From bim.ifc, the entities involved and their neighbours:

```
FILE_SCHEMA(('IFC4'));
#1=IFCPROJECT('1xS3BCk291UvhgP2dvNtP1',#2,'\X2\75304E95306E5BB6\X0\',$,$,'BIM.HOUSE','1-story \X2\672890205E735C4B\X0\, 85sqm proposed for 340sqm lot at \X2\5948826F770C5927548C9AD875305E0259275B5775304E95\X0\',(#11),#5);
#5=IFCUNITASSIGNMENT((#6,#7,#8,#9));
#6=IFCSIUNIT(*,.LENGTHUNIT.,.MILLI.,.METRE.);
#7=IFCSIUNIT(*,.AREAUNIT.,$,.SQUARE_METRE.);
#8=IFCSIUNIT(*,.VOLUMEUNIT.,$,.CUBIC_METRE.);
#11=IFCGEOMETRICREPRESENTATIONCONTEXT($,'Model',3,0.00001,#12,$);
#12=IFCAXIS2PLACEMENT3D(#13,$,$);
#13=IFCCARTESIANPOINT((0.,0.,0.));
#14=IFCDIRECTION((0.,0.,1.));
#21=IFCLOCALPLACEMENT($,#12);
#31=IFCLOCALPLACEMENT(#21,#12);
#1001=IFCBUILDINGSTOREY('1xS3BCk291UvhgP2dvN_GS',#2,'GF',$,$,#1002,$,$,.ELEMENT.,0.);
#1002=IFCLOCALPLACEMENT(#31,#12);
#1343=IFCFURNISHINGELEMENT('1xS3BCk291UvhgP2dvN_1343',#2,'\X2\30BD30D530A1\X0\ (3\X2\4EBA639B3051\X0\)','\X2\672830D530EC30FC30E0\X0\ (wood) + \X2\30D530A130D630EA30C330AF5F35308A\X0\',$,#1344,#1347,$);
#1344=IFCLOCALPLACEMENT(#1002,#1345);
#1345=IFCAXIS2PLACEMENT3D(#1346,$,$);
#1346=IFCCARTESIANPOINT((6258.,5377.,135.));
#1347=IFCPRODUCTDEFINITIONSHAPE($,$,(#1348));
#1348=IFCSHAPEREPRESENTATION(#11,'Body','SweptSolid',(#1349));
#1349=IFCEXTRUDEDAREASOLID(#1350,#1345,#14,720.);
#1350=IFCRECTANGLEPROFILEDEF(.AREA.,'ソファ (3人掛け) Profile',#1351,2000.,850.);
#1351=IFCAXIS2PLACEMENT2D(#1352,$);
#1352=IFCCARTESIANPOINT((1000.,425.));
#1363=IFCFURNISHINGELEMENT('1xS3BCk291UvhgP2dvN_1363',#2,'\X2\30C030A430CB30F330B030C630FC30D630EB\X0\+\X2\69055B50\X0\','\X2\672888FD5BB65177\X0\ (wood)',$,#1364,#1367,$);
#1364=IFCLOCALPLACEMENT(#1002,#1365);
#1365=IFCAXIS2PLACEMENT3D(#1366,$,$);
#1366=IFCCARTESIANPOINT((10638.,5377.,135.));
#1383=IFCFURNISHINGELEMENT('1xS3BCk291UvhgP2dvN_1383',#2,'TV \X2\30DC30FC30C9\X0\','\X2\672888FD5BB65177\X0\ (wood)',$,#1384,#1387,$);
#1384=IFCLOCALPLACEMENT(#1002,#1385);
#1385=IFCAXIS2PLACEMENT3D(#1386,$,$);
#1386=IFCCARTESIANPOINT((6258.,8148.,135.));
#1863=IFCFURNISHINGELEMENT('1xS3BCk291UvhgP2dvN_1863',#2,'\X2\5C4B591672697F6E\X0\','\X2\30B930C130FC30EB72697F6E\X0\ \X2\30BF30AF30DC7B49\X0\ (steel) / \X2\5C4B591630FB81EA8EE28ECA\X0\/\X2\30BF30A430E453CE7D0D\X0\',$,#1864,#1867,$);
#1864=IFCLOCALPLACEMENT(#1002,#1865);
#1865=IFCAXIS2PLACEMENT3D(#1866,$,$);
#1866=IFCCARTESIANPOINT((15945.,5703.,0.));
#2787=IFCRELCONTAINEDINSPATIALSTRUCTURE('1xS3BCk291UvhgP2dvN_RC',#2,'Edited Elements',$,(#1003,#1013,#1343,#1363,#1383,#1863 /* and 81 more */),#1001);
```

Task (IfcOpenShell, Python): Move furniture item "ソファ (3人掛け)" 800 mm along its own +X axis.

```python
import ifcopenshell
import ifcopenshell.api.geometry
import ifcopenshell.util.placement
import ifcopenshell.util.unit

model = ifcopenshell.open("bim.ifc")
unit_scale = ifcopenshell.util.unit.calculate_unit_scale(model)

item = model.by_guid("1xS3BCk291UvhgP2dvN_1343")
matrix = ifcopenshell.util.placement.get_local_placement(item.ObjectPlacement)
matrix[:3, 3] += matrix[:3, 0] * 0.8 / unit_scale
ifcopenshell.api.geometry.edit_object_placement(model, product=item, matrix=matrix, is_si=False)

print(ifcopenshell.util.placement.get_local_placement(item.ObjectPlacement).round(3) + 0.0)

model.write("bim_updated.ifc")
```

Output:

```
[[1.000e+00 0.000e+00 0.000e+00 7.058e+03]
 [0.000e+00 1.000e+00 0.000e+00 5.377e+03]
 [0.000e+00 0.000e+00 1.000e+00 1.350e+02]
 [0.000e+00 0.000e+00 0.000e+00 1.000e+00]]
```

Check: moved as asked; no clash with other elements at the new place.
